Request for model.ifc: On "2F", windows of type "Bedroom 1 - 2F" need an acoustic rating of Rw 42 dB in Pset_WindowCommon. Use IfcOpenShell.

First a look at what the model holds.

```python
import ifcopenshell
import ifcopenshell.util.element

model = ifcopenshell.open("model.ifc")
print(model.schema)
storey = next(s for s in model.by_type("IfcBuildingStorey") if s.Name == "2F")
windows = [e for e in ifcopenshell.util.element.get_decomposition(storey) if e.is_a("IfcWindow")]
seen = {}
for e in windows:
    element_type = ifcopenshell.util.element.get_type(e)
    key = (element_type.Name if element_type != e and element_type else None, ifcopenshell.util.element.get_pset(e, "Pset_WindowCommon", "AcousticRating"))
    seen[key] = seen.get(key, 0) + 1
for (name, value), count in sorted(seen.items(), key=str):
    print(count, "x", name, "|", value)
```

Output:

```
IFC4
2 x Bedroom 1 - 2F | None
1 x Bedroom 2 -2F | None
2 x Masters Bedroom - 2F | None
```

```python
import ifcopenshell
import ifcopenshell.api.pset
import ifcopenshell.util.element

model = ifcopenshell.open("model.ifc")

storey = next(s for s in model.by_type("IfcBuildingStorey") if s.Name == "2F")
windows = [e for e in ifcopenshell.util.element.get_decomposition(storey) if e.is_a("IfcWindow")]

count = 0
for e in windows:
    element_type = ifcopenshell.util.element.get_type(e)
    if element_type in (None, e) or element_type.Name != "Bedroom 1 - 2F":
        continue
    # add_pset returns the element's existing set when there is one.
    pset = ifcopenshell.api.pset.add_pset(model, product=e, name="Pset_WindowCommon")
    ifcopenshell.api.pset.edit_pset(model, pset=pset, properties={"AcousticRating": "Rw 42 dB"})
    count += 1

print(count, "windows updated")

model.write("model-out.ifc")
```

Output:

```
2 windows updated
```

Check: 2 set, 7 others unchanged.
